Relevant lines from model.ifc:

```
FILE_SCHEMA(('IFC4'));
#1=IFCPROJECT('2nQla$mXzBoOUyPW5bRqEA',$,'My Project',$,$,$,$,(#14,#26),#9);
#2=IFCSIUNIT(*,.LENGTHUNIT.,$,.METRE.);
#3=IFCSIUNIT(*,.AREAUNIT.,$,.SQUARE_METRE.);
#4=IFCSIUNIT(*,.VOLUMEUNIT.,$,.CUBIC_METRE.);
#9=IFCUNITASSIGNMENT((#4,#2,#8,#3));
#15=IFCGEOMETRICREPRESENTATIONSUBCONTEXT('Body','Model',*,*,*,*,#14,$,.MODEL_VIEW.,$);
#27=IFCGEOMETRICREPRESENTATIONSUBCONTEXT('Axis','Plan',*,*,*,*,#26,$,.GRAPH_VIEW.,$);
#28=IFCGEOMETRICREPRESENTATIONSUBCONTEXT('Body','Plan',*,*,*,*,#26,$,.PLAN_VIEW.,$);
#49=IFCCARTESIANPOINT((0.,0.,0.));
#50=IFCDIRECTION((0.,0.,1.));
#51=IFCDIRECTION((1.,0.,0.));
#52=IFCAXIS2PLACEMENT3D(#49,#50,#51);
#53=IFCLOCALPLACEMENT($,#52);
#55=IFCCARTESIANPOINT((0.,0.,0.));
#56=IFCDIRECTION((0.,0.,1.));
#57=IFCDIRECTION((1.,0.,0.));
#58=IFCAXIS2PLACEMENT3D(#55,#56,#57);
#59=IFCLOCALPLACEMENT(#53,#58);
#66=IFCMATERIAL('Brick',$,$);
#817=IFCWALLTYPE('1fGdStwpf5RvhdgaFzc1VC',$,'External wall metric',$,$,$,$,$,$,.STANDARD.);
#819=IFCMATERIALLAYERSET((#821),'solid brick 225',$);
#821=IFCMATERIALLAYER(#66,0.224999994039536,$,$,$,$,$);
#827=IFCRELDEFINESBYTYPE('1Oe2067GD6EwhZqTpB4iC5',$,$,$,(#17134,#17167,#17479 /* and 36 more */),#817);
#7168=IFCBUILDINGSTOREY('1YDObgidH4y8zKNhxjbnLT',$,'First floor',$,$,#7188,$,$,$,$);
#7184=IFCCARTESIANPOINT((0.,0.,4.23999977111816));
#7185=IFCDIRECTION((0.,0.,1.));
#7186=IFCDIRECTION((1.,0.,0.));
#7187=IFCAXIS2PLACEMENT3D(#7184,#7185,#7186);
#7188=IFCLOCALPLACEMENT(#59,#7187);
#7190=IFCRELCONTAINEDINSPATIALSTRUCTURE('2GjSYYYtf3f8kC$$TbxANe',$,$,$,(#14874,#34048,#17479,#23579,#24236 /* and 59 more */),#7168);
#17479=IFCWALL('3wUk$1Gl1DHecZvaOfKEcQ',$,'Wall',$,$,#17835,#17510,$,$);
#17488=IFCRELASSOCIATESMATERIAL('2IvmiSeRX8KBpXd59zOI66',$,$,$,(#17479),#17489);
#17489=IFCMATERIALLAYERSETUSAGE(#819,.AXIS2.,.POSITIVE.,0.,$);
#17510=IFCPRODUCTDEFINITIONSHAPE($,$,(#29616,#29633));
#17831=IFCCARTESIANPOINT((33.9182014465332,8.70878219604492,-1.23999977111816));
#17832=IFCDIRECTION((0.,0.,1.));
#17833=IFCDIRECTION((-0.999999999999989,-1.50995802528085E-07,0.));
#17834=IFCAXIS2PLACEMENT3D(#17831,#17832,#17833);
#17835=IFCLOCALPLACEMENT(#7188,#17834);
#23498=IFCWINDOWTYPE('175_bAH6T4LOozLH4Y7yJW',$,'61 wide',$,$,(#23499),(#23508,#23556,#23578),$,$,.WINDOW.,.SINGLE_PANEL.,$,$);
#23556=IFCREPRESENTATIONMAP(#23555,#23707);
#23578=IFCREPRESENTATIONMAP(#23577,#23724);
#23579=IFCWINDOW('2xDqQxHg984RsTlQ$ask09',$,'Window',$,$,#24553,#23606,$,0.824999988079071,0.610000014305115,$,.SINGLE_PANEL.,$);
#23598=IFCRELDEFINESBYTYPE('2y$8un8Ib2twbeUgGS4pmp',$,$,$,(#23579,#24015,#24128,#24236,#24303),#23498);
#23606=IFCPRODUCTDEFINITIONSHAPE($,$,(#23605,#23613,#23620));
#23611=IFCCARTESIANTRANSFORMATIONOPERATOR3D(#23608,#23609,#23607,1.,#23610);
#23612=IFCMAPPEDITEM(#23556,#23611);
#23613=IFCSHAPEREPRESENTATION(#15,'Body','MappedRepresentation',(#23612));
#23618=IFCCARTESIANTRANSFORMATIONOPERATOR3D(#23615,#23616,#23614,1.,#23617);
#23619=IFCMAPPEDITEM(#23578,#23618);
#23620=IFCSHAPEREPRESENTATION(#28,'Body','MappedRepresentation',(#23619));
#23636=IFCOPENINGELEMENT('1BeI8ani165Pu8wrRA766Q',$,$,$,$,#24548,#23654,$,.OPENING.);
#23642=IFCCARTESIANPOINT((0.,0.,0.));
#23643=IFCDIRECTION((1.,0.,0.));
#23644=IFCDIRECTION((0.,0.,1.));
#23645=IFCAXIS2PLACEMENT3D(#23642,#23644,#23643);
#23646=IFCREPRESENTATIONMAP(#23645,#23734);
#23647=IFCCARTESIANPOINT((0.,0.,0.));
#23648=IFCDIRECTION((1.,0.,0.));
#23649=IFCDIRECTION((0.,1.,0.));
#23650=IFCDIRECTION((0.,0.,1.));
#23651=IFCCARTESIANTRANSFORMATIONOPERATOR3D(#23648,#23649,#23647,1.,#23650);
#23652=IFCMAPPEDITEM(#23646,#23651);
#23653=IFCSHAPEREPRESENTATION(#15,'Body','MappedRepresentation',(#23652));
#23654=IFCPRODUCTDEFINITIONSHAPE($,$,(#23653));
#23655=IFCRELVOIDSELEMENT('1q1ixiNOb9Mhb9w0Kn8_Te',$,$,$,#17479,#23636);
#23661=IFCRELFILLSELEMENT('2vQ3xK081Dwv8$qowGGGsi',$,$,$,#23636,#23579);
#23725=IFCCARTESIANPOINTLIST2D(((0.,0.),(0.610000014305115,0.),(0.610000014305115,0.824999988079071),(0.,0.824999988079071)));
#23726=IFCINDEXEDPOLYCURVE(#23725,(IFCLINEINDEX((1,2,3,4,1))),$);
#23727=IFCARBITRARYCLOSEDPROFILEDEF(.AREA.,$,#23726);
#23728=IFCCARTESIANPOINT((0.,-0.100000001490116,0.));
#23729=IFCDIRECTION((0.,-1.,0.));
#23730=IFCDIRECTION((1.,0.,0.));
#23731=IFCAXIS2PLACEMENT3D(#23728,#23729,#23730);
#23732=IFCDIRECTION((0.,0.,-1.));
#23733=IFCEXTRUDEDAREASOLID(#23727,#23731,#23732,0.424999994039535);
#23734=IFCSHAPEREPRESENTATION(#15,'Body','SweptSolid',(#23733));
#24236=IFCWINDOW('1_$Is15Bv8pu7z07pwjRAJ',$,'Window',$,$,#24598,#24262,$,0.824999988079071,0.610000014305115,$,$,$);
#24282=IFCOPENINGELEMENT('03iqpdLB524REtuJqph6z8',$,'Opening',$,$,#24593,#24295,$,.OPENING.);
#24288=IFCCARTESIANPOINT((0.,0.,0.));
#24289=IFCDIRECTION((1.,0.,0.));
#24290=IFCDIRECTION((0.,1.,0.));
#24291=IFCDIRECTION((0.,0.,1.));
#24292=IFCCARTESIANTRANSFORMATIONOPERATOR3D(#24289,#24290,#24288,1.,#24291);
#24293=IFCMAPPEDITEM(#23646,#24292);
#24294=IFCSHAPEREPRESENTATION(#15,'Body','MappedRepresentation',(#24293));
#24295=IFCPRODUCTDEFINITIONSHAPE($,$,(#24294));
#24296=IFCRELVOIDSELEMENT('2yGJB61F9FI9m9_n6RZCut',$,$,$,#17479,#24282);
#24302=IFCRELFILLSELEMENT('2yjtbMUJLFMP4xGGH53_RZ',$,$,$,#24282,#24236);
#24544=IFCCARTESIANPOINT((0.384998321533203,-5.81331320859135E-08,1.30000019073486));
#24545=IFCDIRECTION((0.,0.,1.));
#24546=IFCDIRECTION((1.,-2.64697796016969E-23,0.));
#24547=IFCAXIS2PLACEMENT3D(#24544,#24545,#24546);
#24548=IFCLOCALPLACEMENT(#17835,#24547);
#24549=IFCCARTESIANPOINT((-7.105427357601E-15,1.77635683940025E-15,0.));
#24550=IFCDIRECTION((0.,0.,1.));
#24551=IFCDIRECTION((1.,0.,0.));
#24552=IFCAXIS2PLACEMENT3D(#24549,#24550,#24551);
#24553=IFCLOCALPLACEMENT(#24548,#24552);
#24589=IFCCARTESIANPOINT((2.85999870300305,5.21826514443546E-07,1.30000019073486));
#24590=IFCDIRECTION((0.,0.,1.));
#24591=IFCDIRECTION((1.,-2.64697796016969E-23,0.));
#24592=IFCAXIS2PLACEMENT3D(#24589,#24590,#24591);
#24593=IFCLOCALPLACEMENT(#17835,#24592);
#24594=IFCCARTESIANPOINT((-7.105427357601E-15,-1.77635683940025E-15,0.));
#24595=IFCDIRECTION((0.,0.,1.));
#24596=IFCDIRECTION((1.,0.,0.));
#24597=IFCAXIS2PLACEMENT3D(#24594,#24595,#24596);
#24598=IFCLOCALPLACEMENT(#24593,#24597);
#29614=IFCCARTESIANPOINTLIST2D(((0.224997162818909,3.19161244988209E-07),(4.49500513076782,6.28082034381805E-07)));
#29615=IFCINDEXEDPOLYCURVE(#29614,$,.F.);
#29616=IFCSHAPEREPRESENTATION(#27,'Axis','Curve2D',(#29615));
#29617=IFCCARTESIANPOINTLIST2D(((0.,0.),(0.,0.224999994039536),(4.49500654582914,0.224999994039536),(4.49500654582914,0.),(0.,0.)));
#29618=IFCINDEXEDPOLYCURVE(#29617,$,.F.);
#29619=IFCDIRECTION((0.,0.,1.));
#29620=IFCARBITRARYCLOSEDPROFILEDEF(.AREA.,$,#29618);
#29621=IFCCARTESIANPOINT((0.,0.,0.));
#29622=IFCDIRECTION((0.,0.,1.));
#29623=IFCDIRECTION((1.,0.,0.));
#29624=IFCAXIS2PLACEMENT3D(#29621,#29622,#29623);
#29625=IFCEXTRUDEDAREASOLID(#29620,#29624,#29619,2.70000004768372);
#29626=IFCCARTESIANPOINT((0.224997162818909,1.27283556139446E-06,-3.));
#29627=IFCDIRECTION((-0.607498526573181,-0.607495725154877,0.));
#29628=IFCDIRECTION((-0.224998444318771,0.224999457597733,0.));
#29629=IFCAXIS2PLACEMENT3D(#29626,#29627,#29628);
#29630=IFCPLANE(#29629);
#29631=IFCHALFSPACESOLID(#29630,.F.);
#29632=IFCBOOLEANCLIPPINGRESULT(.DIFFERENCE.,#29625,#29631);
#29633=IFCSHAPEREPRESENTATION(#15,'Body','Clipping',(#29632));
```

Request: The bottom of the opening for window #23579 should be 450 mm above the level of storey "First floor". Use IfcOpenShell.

```python
import numpy as np
import ifcopenshell
import ifcopenshell.api.geometry
import ifcopenshell.geom
import ifcopenshell.util.element
import ifcopenshell.util.placement
import ifcopenshell.util.shape
import ifcopenshell.util.unit

model = ifcopenshell.open("model.ifc")
unit_scale = ifcopenshell.util.unit.calculate_unit_scale(model)

window = model.by_id(23579)
opening = window.FillsVoids[0].RelatingOpeningElement
storey = ifcopenshell.util.element.get_container(window, ifc_class="IfcBuildingStorey")
level = ifcopenshell.util.placement.get_local_placement(storey.ObjectPlacement)[2, 3]

# The opening's origin need not be at the sill, so measure its lowest point.
shape = ifcopenshell.geom.create_shape(ifcopenshell.geom.settings(), opening)
bottom = ifcopenshell.util.shape.get_shape_bottom_elevation(shape, shape.geometry) / unit_scale
dz = level + 0.45 / unit_scale - bottom

shift = np.array([0.0, 0.0, dz])
# The window is placed relative to its opening, so it follows when the opening moves.
matrix = ifcopenshell.util.placement.get_local_placement(opening.ObjectPlacement)
matrix[:3, 3] += shift
ifcopenshell.api.geometry.edit_object_placement(
    model, product=opening, matrix=matrix, is_si=False, should_transform_children=True
)

print(f"moved by {dz * unit_scale:+.3f} m")

model.write("model-out.ifc")
```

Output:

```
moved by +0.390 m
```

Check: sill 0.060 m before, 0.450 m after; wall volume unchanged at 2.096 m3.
